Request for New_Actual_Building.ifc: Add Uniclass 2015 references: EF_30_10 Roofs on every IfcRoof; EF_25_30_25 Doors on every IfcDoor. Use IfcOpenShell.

First a look at what the model holds.

```python
import ifcopenshell

model = ifcopenshell.open("New_Actual_Building.ifc")
print(model.schema)
print("classifications:", [c.Name for c in model.by_type("IfcClassification")])
for ifc_class in ("IfcDoor", "IfcRoof", "IfcStair", "IfcWall", "IfcWindow"):
    print(ifc_class, len(model.by_type(ifc_class)))
```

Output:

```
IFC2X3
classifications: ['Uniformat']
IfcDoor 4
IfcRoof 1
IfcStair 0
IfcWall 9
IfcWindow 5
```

```python
import ifcopenshell
import ifcopenshell.api.classification

model = ifcopenshell.open("New_Actual_Building.ifc")

# IFC2X3 requires Source and Edition and has no link from the project to the system.
system = model.create_entity("IfcClassification", Source="NBS", Edition="2015", Name="Uniclass 2015")

codes = {
    "IfcRoof": ("EF_30_10", "Roofs"),
    "IfcDoor": ("EF_25_30_25", "Doors"),
}
for ifc_class, (code, name) in codes.items():
    products = model.by_type(ifc_class)
    ifcopenshell.api.classification.add_reference(
        model, products=products, classification=system, identification=code, name=name
    )
    print(code, len(products))

model.write("New_Actual_Building_edited.ifc")
```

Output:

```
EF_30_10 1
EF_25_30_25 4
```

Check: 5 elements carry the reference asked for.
